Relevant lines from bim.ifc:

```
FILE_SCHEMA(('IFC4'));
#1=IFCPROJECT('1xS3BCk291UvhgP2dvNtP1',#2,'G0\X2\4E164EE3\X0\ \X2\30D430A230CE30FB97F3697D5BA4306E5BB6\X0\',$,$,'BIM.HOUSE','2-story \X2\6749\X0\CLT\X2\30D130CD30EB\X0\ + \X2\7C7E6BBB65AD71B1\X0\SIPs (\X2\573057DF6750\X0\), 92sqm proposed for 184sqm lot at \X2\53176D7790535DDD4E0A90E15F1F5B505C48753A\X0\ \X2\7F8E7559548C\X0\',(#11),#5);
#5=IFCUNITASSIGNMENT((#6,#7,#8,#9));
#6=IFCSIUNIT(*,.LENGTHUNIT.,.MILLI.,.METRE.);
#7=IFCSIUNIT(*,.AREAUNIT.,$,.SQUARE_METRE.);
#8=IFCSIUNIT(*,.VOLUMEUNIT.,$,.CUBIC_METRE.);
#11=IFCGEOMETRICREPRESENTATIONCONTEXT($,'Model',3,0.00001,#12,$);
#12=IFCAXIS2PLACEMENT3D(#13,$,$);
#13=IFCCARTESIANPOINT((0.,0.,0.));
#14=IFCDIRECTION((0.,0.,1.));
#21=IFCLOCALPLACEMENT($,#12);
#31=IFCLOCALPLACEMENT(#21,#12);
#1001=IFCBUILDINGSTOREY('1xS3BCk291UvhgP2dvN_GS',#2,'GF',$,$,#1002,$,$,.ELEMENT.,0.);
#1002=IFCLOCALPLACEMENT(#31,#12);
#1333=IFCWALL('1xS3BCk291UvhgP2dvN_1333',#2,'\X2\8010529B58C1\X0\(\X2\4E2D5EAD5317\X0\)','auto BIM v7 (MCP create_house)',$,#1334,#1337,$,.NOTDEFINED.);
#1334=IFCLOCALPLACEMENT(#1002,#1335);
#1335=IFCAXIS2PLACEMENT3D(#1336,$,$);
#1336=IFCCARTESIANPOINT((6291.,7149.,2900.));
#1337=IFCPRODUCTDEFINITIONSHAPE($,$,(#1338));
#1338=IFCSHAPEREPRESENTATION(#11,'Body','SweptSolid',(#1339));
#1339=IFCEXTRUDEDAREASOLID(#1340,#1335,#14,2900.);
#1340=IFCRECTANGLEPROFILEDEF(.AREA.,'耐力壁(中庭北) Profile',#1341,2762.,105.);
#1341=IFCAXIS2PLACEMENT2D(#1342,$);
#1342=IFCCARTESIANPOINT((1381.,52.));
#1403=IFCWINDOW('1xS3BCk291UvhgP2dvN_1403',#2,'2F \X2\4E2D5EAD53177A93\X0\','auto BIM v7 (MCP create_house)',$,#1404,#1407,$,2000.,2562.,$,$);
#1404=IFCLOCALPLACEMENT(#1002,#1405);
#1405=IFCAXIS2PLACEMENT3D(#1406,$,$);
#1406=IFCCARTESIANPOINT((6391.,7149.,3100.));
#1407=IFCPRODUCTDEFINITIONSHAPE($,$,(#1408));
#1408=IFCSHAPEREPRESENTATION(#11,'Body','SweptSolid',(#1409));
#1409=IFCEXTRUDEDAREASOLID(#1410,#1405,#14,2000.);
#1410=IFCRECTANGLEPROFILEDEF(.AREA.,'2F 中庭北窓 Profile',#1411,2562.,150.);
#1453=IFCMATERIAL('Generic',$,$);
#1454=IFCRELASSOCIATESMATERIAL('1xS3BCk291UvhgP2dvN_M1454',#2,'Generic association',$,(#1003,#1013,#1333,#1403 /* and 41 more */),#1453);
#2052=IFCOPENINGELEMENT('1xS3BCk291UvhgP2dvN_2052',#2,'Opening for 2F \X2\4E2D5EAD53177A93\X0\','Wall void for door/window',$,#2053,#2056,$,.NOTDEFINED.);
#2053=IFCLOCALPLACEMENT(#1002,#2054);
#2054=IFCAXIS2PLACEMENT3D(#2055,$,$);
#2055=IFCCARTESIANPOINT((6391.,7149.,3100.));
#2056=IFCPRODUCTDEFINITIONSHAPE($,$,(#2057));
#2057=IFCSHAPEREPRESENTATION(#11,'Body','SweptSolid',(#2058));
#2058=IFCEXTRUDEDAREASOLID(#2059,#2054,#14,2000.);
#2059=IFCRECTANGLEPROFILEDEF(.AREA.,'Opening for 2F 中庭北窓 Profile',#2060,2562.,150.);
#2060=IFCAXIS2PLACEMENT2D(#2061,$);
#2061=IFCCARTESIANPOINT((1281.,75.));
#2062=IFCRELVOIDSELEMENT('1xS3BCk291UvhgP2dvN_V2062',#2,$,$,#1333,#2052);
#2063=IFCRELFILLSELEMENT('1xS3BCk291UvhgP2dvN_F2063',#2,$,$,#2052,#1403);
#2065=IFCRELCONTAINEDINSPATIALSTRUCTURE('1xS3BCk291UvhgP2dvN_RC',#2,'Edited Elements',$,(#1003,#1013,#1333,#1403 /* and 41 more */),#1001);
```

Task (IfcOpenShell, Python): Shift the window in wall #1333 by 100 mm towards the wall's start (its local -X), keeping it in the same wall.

```python
import ifcopenshell
import ifcopenshell.api.geometry
import ifcopenshell.util.placement
import ifcopenshell.util.unit

model = ifcopenshell.open("bim.ifc")
unit_scale = ifcopenshell.util.unit.calculate_unit_scale(model)

window = model.by_guid("1xS3BCk291UvhgP2dvN_1403")
opening = window.FillsVoids[0].RelatingOpeningElement
wall = opening.VoidsElements[0].RelatingBuildingElement

wall_matrix = ifcopenshell.util.placement.get_local_placement(wall.ObjectPlacement)
shift = wall_matrix[:3, 0] * -0.1 / unit_scale
before = ifcopenshell.util.placement.get_local_placement(window.ObjectPlacement)[:3, 3].copy()

# The window is not placed relative to its opening, so move both.
for product in (opening, window):
    matrix = ifcopenshell.util.placement.get_local_placement(product.ObjectPlacement)
    matrix[:3, 3] += shift
    ifcopenshell.api.geometry.edit_object_placement(model, product=product, matrix=matrix, is_si=False)

after = ifcopenshell.util.placement.get_local_placement(window.ObjectPlacement)[:3, 3]
print("window moved by", (after - before).round(3) + 0.0)

model.write("bim_edited.ifc")
```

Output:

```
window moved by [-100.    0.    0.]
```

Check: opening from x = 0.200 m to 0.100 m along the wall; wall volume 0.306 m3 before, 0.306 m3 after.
